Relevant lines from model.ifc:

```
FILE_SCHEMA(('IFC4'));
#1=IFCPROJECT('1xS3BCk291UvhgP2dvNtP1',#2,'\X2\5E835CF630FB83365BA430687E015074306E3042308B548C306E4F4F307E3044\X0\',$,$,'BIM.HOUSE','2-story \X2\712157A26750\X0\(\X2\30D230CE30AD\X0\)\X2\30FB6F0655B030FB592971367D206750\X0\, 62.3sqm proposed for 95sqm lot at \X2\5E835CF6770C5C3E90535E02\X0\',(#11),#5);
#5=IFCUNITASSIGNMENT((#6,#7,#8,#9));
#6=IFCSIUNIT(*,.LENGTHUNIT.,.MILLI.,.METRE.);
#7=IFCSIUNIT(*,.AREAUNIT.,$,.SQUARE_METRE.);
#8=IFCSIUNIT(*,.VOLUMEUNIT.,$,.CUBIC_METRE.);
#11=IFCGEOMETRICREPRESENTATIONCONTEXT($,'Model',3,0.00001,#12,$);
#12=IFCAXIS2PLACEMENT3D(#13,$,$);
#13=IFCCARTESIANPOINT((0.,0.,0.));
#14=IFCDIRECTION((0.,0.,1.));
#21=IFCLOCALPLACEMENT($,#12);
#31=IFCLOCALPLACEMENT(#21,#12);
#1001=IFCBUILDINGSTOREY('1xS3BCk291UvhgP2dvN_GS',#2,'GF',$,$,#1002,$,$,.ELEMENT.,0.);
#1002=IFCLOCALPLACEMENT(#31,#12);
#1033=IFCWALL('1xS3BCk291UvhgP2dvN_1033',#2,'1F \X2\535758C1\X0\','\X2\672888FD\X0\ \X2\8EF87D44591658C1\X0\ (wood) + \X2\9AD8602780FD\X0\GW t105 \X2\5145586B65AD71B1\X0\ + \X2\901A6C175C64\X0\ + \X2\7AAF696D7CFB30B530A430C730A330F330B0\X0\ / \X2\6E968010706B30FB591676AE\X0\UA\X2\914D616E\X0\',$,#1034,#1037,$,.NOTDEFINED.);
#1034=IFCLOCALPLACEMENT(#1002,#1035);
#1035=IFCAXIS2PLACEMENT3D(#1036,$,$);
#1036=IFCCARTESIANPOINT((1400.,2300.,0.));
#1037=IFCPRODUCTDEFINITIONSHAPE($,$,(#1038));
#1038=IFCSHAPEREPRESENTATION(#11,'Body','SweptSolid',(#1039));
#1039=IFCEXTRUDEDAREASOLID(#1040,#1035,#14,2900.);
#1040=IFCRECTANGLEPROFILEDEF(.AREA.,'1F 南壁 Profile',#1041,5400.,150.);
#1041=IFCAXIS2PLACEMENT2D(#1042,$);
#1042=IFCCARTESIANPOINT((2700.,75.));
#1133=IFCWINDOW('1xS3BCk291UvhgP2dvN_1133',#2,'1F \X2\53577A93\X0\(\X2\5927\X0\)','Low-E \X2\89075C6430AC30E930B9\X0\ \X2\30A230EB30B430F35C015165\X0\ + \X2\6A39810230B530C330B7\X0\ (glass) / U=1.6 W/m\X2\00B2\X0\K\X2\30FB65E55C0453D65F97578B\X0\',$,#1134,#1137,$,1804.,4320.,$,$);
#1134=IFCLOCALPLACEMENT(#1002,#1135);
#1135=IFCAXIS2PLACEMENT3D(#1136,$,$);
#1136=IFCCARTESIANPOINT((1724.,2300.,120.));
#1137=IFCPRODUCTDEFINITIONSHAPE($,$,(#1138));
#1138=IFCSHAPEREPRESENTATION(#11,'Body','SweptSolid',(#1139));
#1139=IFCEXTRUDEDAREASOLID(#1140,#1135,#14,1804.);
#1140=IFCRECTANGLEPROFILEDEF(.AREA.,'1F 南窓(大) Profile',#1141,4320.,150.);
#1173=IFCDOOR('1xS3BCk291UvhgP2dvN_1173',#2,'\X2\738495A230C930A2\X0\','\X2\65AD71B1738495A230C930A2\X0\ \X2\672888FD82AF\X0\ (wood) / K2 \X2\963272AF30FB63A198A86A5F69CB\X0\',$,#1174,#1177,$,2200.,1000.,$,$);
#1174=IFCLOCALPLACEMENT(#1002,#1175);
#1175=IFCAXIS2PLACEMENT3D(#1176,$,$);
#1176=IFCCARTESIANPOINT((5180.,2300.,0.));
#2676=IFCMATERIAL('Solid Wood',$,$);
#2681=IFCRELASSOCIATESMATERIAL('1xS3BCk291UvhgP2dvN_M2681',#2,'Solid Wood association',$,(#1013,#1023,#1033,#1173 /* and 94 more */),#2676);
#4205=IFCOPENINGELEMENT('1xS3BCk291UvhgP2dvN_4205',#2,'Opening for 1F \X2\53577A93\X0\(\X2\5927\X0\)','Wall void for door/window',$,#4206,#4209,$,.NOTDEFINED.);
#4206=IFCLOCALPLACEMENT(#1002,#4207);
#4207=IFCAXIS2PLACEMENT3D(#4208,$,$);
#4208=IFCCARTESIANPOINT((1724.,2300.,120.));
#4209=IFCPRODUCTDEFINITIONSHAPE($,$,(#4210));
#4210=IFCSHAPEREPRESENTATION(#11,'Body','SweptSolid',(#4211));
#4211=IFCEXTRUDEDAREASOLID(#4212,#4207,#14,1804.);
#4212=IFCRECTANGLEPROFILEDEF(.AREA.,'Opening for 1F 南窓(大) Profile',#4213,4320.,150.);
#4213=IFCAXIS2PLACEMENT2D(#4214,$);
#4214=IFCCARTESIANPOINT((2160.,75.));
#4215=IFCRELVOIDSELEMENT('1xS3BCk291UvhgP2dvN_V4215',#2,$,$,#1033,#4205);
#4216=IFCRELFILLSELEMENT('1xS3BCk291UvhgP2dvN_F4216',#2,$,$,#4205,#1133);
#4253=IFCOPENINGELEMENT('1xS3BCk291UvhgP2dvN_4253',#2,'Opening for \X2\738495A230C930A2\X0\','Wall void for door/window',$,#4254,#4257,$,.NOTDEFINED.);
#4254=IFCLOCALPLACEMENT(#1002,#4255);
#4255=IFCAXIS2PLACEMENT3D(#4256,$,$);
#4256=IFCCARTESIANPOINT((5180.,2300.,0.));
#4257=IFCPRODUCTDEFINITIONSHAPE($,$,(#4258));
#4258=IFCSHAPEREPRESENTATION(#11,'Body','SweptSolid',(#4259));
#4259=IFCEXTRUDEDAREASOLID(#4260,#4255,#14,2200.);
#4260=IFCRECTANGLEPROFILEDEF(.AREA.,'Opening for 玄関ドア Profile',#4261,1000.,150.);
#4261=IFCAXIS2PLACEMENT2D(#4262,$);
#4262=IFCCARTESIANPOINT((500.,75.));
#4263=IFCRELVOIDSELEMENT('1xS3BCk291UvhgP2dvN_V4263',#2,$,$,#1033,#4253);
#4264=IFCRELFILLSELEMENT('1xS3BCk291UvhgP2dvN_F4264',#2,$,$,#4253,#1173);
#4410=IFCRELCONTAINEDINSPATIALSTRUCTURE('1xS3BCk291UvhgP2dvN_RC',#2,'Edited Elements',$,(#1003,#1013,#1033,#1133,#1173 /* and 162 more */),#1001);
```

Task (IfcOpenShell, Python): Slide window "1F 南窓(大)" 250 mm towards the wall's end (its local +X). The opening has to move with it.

```python
import ifcopenshell
import ifcopenshell.api.geometry
import ifcopenshell.util.placement
import ifcopenshell.util.unit

model = ifcopenshell.open("model.ifc")
unit_scale = ifcopenshell.util.unit.calculate_unit_scale(model)

window = model.by_guid("1xS3BCk291UvhgP2dvN_1133")
opening = window.FillsVoids[0].RelatingOpeningElement
wall = opening.VoidsElements[0].RelatingBuildingElement

wall_matrix = ifcopenshell.util.placement.get_local_placement(wall.ObjectPlacement)
shift = wall_matrix[:3, 0] * 0.25 / unit_scale
before = ifcopenshell.util.placement.get_local_placement(window.ObjectPlacement)[:3, 3].copy()

# The window is not placed relative to its opening, so move both.
for product in (opening, window):
    matrix = ifcopenshell.util.placement.get_local_placement(product.ObjectPlacement)
    matrix[:3, 3] += shift
    ifcopenshell.api.geometry.edit_object_placement(model, product=product, matrix=matrix, is_si=False)

after = ifcopenshell.util.placement.get_local_placement(window.ObjectPlacement)[:3, 3]
print("window moved by", (after - before).round(3) + 0.0)

model.write("model_updated.ifc")
```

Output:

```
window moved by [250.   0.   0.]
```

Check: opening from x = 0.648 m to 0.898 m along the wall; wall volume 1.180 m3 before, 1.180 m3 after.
